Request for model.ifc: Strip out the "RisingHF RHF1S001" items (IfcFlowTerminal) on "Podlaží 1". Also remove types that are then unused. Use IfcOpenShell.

First a look at what the model holds.

```python
import ifcopenshell
import ifcopenshell.util.element

model = ifcopenshell.open("model.ifc")
print(model.schema)
storey = next(s for s in model.by_type("IfcBuildingStorey") if s.Name == "Podlaží 1")
terminals = [e for e in ifcopenshell.util.element.get_decomposition(storey) if e.is_a("IfcFlowTerminal")]
seen = {}
for e in terminals:
    element_type = ifcopenshell.util.element.get_type(e)
    name = element_type.Name if element_type not in (None, e) else None
    seen[name] = seen.get(name, 0) + 1
for name, count in sorted(seen.items(), key=str):
    print(count, "x", name)
```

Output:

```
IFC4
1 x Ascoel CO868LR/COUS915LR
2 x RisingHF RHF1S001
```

```python
import ifcopenshell
import ifcopenshell.api.root
import ifcopenshell.util.element

model = ifcopenshell.open("model.ifc")

storey = next(s for s in model.by_type("IfcBuildingStorey") if s.Name == "Podlaží 1")
terminals = [e for e in ifcopenshell.util.element.get_decomposition(storey) if e.is_a("IfcFlowTerminal")]
targets = [e for e in terminals if (t := ifcopenshell.util.element.get_type(e)) not in (None, e) and t.Name == "RisingHF RHF1S001"]
types = {ifcopenshell.util.element.get_type(e) for e in targets} - {None, *targets}

for e in targets:
    ifcopenshell.api.root.remove_product(model, product=e)
print(len(targets), "removed")

unused = [t for t in types if not ifcopenshell.util.element.get_types(t)]
for t in unused:
    ifcopenshell.api.root.remove_product(model, product=t)
print(len(unused), "unused types removed")

model.write("model_updated.ifc")
```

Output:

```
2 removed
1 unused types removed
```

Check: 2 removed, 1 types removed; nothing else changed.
